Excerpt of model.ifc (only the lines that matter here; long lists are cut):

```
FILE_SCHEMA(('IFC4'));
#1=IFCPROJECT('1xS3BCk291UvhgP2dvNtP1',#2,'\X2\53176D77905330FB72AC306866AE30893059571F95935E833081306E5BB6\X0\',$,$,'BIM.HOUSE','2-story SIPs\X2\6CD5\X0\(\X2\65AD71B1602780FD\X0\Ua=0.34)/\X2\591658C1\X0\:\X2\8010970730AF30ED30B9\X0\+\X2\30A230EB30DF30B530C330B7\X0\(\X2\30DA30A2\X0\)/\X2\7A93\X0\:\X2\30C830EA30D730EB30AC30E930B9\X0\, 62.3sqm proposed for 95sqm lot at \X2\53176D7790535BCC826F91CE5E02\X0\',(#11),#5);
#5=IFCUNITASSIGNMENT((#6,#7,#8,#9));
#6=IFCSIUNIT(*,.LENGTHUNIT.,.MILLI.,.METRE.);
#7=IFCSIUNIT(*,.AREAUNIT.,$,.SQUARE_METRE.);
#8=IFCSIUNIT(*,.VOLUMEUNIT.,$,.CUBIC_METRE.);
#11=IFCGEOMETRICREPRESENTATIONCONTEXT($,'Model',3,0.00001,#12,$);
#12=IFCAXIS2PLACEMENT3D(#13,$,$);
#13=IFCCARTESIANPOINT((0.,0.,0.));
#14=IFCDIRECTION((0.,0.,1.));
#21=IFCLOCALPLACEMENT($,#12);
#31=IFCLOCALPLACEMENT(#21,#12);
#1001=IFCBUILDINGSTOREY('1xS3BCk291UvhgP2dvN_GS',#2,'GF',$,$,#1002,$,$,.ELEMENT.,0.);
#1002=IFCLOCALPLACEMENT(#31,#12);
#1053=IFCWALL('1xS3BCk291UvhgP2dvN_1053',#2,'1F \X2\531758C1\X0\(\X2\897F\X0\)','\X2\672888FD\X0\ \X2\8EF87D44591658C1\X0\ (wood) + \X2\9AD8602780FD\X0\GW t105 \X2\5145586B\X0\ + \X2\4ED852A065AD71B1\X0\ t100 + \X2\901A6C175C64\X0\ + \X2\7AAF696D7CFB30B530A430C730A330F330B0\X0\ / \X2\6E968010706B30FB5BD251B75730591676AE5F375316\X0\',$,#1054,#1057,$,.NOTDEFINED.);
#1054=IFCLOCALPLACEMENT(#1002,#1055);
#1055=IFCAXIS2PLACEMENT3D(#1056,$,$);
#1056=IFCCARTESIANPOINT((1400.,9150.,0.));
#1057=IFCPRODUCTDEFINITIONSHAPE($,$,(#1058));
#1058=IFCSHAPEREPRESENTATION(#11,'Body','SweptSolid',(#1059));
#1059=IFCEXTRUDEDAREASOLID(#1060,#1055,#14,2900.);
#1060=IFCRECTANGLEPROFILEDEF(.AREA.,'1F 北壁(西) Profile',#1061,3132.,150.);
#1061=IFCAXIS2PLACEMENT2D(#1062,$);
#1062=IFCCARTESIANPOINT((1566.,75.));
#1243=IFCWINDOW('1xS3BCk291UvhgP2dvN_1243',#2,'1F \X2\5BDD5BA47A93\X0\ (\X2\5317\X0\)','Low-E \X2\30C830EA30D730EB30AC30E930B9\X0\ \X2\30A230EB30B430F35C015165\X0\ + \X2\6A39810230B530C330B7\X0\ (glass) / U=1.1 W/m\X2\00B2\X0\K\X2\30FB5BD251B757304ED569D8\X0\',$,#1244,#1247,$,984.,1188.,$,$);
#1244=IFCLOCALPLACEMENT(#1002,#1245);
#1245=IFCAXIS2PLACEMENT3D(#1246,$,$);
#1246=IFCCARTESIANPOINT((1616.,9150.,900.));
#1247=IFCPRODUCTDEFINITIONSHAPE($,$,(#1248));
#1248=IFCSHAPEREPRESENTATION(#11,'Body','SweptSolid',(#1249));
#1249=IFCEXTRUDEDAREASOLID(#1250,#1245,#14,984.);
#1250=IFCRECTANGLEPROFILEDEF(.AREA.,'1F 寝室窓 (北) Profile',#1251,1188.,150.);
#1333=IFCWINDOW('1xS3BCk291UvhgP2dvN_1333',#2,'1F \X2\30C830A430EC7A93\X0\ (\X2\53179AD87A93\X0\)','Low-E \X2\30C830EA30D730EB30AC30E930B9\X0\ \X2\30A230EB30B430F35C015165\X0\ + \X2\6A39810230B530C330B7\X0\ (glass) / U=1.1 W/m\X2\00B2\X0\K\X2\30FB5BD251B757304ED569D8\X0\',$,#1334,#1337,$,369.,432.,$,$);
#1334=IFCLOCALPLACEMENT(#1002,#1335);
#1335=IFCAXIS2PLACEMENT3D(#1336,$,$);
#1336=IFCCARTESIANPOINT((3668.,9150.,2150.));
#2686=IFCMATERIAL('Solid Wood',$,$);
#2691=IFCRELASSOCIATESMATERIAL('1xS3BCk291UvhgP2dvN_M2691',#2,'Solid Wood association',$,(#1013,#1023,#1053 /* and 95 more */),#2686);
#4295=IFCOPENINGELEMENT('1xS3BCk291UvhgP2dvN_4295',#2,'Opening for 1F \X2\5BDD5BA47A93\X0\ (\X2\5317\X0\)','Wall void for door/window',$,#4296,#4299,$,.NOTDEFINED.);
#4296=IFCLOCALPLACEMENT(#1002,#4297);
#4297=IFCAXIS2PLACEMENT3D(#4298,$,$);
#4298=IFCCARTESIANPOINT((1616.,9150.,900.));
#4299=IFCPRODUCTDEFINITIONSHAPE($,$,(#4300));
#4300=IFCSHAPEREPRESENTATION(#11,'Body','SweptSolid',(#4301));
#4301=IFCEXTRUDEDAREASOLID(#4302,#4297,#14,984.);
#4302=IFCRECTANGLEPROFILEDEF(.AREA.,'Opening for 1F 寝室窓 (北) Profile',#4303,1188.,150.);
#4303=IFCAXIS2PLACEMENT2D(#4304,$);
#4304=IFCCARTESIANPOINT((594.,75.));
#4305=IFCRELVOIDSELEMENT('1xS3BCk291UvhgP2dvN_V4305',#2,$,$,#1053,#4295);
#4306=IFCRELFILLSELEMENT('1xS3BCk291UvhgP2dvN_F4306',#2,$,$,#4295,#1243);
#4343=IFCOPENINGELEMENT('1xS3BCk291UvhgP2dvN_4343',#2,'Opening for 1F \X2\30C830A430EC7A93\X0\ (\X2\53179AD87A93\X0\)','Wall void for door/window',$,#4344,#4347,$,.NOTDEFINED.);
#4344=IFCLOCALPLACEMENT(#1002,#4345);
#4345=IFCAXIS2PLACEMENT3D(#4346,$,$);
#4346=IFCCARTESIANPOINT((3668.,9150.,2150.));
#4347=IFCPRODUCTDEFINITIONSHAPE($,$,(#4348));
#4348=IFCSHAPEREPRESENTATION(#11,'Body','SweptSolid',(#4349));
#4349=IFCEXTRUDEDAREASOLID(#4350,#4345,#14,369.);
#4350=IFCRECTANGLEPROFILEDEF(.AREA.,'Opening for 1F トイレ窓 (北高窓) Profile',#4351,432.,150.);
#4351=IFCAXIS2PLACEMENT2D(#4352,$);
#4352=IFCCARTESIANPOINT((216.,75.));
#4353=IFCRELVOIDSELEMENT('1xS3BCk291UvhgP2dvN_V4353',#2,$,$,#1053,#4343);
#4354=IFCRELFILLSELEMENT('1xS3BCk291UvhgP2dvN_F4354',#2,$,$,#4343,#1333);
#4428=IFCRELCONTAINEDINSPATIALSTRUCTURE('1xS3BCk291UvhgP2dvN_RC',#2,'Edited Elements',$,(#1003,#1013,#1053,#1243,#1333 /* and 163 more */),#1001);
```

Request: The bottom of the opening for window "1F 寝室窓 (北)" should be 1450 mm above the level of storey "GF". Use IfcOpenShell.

```python
import numpy as np
import ifcopenshell
import ifcopenshell.api.geometry
import ifcopenshell.geom
import ifcopenshell.util.element
import ifcopenshell.util.placement
import ifcopenshell.util.shape
import ifcopenshell.util.unit

model = ifcopenshell.open("model.ifc")
unit_scale = ifcopenshell.util.unit.calculate_unit_scale(model)

window = model.by_guid("1xS3BCk291UvhgP2dvN_1243")
opening = window.FillsVoids[0].RelatingOpeningElement
storey = ifcopenshell.util.element.get_container(window, ifc_class="IfcBuildingStorey")
level = ifcopenshell.util.placement.get_local_placement(storey.ObjectPlacement)[2, 3]

# The opening's origin need not be at the sill, so measure its lowest point.
shape = ifcopenshell.geom.create_shape(ifcopenshell.geom.settings(), opening)
bottom = ifcopenshell.util.shape.get_shape_bottom_elevation(shape, shape.geometry) / unit_scale
dz = level + 1450.0 - bottom

shift = np.array([0.0, 0.0, dz])
# The window is not placed relative to its opening, so move both.
for product in (opening, window):
    matrix = ifcopenshell.util.placement.get_local_placement(product.ObjectPlacement)
    matrix[:3, 3] += shift
    ifcopenshell.api.geometry.edit_object_placement(model, product=product, matrix=matrix, is_si=False)

print(f"moved by {dz * unit_scale:+.3f} m")

model.write("model_rev.ifc")
```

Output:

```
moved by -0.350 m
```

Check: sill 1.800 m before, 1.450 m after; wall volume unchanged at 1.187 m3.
